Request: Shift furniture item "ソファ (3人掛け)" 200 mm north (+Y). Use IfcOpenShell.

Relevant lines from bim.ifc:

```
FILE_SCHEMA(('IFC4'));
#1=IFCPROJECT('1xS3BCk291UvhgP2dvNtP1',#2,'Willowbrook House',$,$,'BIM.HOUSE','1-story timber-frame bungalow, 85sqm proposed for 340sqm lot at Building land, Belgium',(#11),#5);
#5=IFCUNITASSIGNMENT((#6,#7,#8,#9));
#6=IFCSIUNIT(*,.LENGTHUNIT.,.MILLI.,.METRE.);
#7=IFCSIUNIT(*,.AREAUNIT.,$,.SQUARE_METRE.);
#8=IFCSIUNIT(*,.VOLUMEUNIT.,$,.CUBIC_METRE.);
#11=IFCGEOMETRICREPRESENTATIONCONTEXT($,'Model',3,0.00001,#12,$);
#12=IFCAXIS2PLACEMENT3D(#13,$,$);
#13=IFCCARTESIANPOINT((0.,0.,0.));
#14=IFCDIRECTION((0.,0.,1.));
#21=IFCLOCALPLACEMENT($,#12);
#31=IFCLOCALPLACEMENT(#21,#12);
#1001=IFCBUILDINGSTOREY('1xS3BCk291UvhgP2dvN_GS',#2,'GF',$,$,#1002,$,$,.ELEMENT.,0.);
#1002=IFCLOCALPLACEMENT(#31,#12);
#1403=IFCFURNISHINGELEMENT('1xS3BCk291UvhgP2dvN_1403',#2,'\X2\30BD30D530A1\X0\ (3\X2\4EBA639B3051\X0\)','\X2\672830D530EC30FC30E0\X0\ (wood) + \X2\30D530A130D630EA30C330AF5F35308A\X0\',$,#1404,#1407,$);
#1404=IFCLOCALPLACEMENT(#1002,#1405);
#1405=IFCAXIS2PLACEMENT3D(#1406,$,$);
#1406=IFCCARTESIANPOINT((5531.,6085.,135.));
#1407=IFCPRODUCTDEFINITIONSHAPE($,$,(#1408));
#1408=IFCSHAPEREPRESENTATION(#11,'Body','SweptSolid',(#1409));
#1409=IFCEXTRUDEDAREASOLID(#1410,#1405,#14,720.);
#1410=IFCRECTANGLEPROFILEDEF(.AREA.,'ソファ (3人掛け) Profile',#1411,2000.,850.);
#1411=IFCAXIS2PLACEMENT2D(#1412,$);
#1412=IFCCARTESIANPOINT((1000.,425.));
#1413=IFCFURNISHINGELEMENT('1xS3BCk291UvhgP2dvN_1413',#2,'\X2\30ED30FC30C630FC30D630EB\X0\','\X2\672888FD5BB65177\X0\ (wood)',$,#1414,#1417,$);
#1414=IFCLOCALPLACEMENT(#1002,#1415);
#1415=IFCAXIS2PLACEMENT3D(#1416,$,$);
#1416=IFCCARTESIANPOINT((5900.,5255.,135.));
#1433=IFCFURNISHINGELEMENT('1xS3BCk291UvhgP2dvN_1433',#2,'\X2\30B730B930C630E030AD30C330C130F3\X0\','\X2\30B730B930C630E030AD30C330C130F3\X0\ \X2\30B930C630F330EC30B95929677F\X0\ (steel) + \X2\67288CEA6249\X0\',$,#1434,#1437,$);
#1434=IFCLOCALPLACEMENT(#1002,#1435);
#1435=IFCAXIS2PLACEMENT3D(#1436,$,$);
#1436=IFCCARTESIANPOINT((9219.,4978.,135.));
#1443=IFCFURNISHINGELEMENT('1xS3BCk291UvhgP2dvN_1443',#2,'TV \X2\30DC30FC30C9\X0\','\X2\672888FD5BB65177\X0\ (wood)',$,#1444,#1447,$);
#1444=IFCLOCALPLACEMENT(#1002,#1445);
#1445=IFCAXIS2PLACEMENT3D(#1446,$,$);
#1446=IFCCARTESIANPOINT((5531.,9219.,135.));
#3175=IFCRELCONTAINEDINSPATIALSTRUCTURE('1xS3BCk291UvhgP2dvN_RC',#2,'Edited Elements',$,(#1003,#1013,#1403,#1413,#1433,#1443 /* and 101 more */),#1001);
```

```python
import ifcopenshell
import ifcopenshell.api.geometry
import ifcopenshell.util.placement

model = ifcopenshell.open("bim.ifc")

item = model.by_guid("1xS3BCk291UvhgP2dvN_1403")
matrix = ifcopenshell.util.placement.get_local_placement(item.ObjectPlacement)
matrix[1, 3] += 200.0
ifcopenshell.api.geometry.edit_object_placement(model, product=item, matrix=matrix, is_si=False)

print(ifcopenshell.util.placement.get_local_placement(item.ObjectPlacement).round(3) + 0.0)

model.write("bim_edited.ifc")
```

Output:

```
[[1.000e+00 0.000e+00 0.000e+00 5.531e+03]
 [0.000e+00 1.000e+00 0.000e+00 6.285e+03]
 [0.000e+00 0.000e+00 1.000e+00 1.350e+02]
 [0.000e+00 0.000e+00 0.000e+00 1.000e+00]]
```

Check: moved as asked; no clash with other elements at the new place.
